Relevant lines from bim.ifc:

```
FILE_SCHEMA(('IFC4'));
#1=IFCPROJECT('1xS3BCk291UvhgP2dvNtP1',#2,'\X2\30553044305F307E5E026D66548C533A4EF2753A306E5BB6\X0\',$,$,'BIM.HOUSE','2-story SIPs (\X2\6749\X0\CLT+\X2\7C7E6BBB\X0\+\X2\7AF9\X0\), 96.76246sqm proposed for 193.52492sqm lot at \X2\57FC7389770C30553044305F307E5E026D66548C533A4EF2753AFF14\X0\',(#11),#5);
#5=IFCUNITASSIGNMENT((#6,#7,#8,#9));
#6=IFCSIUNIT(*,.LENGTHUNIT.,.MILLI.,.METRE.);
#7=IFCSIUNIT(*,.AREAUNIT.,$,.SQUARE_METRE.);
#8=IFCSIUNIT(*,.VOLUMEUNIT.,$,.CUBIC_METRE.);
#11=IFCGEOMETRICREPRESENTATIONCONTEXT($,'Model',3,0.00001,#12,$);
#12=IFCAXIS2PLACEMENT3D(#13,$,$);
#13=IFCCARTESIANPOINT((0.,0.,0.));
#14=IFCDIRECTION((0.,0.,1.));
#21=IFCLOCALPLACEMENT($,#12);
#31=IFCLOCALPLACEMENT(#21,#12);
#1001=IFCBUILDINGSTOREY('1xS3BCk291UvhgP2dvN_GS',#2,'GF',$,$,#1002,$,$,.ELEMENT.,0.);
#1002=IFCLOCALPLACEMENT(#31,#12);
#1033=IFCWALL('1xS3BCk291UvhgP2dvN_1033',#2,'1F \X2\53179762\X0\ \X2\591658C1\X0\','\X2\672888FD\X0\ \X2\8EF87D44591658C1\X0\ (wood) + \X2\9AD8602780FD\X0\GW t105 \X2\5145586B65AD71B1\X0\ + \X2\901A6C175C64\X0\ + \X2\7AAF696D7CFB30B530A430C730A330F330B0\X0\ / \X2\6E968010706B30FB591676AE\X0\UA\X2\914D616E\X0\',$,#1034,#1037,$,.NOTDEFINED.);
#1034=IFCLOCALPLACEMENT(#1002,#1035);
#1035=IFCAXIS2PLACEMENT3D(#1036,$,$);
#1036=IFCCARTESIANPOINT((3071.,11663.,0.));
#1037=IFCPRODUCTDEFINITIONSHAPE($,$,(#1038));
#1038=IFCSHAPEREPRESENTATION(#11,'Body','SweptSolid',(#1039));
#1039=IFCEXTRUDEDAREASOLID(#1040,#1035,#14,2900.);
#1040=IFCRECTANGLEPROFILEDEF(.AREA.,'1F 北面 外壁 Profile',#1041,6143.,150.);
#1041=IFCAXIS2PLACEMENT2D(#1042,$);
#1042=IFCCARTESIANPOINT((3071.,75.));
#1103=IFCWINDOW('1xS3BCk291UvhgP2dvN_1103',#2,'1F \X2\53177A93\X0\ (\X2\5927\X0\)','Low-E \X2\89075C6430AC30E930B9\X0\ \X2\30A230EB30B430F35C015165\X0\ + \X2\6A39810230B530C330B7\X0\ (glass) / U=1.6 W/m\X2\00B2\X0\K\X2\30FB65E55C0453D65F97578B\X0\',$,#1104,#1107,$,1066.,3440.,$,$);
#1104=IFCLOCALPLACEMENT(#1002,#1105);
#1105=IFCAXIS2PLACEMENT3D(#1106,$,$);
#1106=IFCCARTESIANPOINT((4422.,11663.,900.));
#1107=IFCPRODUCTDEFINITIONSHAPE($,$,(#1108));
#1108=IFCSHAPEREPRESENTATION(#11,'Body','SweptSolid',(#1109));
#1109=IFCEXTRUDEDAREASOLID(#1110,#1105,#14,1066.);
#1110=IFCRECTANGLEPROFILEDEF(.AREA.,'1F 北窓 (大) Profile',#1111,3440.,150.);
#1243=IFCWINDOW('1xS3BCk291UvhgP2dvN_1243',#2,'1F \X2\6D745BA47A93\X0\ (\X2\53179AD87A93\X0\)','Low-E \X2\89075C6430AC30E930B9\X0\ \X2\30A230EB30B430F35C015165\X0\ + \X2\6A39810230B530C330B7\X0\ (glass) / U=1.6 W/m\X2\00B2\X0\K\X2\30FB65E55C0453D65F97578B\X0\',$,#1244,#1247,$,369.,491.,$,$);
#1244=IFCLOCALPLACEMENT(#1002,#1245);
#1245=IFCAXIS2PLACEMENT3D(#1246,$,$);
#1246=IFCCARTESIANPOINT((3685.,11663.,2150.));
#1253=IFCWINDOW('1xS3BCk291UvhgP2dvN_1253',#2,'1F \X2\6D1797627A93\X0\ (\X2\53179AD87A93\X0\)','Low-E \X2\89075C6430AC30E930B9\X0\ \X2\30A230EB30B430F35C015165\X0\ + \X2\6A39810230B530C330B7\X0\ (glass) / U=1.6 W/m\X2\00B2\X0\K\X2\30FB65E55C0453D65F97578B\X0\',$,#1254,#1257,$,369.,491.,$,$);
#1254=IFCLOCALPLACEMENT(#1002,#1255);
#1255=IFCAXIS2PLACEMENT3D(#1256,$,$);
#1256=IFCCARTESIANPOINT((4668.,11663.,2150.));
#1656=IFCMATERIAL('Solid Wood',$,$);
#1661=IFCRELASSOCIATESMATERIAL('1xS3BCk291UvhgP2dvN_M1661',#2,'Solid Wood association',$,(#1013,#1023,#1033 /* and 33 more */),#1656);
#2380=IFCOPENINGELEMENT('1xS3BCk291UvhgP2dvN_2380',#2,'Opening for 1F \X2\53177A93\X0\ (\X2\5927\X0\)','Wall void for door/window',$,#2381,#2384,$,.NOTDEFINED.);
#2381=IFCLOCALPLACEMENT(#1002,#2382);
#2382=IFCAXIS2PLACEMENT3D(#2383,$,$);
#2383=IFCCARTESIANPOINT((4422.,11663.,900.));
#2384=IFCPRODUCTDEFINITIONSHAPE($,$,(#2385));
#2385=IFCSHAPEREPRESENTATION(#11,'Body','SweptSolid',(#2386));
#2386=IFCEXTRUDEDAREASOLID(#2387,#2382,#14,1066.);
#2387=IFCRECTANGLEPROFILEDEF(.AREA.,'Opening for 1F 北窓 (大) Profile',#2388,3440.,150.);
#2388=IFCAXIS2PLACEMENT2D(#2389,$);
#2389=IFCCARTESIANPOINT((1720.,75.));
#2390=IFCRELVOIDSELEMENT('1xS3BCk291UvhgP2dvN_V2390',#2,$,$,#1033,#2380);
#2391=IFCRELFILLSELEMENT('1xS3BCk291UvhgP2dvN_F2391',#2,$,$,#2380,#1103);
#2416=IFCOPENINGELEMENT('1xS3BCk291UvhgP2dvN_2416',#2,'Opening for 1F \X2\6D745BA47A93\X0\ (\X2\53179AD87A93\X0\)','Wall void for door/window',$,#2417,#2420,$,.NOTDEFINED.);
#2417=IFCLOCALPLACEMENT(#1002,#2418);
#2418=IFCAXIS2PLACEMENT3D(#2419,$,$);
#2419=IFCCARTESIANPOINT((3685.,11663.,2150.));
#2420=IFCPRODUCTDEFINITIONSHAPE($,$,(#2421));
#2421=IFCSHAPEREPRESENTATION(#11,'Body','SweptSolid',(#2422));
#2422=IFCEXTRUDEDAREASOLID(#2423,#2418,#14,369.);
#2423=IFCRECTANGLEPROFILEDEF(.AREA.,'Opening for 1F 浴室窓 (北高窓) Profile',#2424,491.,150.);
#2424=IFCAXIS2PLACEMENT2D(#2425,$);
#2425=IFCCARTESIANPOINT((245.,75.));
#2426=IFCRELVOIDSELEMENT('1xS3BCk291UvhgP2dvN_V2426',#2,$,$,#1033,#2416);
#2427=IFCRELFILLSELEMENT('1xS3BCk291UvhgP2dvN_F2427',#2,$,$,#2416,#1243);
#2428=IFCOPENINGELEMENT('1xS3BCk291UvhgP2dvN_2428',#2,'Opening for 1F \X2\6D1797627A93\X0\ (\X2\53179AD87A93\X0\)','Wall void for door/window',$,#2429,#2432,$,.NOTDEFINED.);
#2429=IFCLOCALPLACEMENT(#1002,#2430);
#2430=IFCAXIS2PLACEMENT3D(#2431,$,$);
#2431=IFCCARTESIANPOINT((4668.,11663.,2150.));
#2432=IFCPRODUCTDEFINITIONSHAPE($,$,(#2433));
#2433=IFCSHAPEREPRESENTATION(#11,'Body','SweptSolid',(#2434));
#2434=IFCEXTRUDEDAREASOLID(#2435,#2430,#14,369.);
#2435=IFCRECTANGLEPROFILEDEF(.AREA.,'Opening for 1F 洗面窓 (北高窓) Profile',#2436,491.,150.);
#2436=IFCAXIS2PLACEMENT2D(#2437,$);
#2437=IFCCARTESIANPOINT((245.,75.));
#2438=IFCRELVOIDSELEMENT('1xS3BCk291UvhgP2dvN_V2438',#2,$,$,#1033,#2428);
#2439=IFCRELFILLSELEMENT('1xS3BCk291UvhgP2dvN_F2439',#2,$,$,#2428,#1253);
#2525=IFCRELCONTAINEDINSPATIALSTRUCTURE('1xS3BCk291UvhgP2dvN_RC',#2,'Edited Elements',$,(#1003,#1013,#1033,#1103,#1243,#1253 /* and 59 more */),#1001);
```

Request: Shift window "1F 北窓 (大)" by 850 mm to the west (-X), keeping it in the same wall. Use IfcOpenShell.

```python
import ifcopenshell
import ifcopenshell.api.geometry
import ifcopenshell.util.placement
import ifcopenshell.util.unit

model = ifcopenshell.open("bim.ifc")
unit_scale = ifcopenshell.util.unit.calculate_unit_scale(model)

window = model.by_guid("1xS3BCk291UvhgP2dvN_1103")
opening = window.FillsVoids[0].RelatingOpeningElement
wall = opening.VoidsElements[0].RelatingBuildingElement

wall_matrix = ifcopenshell.util.placement.get_local_placement(wall.ObjectPlacement)
shift = wall_matrix[:3, 0] * -0.85 / unit_scale
before = ifcopenshell.util.placement.get_local_placement(window.ObjectPlacement)[:3, 3].copy()

# The window is not placed relative to its opening, so move both.
for product in (opening, window):
    matrix = ifcopenshell.util.placement.get_local_placement(product.ObjectPlacement)
    matrix[:3, 3] += shift
    ifcopenshell.api.geometry.edit_object_placement(model, product=product, matrix=matrix, is_si=False)

after = ifcopenshell.util.placement.get_local_placement(window.ObjectPlacement)[:3, 3]
print("window moved by", (after - before).round(3) + 0.0)

model.write("bim_updated.ifc")
```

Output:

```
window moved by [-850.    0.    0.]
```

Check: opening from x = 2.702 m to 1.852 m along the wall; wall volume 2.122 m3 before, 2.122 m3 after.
